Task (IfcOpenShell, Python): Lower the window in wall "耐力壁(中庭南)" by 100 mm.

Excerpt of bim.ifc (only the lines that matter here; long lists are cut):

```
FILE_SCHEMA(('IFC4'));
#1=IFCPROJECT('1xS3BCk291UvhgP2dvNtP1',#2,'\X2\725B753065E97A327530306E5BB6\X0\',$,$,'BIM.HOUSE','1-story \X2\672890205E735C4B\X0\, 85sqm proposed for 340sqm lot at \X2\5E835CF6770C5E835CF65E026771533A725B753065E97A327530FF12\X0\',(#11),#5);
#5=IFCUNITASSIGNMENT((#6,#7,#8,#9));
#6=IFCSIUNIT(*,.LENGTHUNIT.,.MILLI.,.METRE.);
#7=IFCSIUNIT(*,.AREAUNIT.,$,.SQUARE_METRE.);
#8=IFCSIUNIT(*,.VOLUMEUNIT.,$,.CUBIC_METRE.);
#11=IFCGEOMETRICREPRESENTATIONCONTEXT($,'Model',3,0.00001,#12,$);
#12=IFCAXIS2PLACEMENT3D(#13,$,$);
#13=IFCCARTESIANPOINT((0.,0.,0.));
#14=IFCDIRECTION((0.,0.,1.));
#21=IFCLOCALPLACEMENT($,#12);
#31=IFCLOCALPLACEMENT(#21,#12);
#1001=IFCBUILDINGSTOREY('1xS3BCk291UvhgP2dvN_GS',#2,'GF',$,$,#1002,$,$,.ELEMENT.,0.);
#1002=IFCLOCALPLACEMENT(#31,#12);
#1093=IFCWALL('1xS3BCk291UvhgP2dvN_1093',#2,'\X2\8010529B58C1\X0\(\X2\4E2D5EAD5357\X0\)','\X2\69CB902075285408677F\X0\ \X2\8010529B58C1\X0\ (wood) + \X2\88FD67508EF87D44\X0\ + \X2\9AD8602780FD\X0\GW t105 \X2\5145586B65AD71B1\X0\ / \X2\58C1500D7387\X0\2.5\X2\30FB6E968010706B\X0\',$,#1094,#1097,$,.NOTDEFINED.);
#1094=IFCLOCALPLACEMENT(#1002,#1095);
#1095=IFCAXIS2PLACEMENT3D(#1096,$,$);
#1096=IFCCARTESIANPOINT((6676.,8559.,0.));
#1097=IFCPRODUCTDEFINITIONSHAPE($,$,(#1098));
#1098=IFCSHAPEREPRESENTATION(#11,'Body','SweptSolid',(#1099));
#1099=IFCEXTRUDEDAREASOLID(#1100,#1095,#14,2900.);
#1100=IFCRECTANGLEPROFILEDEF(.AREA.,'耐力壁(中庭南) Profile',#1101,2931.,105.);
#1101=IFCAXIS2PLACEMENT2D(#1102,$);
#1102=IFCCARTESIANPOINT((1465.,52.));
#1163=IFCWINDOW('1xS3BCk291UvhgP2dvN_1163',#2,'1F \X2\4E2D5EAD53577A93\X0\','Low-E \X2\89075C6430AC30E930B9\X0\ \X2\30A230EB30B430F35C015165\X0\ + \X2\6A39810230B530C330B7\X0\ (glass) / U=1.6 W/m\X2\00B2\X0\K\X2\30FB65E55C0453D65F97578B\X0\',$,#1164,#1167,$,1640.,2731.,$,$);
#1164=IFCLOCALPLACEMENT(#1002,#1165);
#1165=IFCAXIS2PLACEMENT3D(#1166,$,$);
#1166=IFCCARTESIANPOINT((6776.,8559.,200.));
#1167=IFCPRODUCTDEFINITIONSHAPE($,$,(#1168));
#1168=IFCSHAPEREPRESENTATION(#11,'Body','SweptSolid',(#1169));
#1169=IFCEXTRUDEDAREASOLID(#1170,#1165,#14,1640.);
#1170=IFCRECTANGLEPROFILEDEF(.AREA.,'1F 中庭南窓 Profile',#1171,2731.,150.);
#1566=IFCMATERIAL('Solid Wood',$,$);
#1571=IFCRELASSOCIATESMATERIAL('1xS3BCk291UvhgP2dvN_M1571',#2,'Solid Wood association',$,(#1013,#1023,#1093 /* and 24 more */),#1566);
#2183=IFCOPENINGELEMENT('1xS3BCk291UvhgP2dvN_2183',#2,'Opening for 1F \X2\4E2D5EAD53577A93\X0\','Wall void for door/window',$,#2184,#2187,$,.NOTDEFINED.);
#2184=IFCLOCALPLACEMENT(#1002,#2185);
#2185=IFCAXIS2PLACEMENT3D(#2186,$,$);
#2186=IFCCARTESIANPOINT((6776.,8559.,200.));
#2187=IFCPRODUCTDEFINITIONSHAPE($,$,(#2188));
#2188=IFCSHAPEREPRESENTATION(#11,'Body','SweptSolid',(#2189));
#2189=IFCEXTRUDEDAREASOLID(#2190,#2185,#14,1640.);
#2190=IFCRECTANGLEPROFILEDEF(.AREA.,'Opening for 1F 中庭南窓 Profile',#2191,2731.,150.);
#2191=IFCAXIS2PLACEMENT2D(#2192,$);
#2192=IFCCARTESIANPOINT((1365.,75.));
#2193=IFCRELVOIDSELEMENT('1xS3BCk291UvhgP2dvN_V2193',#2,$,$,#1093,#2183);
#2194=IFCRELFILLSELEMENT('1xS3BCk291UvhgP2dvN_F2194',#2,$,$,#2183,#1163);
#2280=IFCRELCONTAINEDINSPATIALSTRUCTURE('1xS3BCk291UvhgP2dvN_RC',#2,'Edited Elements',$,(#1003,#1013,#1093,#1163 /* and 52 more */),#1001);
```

```python
import numpy as np
import ifcopenshell
import ifcopenshell.api.geometry
import ifcopenshell.util.placement
import ifcopenshell.util.unit

model = ifcopenshell.open("bim.ifc")
unit_scale = ifcopenshell.util.unit.calculate_unit_scale(model)

window = model.by_guid("1xS3BCk291UvhgP2dvN_1163")
opening = window.FillsVoids[0].RelatingOpeningElement
dz = -0.1 / unit_scale

shift = np.array([0.0, 0.0, dz])
# The window is not placed relative to its opening, so move both.
for product in (opening, window):
    matrix = ifcopenshell.util.placement.get_local_placement(product.ObjectPlacement)
    matrix[:3, 3] += shift
    ifcopenshell.api.geometry.edit_object_placement(model, product=product, matrix=matrix, is_si=False)

print(f"moved by {dz * unit_scale:+.3f} m")

model.write("bim_updated.ifc")
```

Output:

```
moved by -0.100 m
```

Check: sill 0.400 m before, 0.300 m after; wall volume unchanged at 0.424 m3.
